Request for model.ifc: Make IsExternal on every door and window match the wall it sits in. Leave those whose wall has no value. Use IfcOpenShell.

First a look at what the model holds.

```python
import ifcopenshell
import ifcopenshell.util.element

model = ifcopenshell.open("model.ifc")
print(model.schema)
seen = {}
for e in model.by_type("IfcDoor") + model.by_type("IfcWindow"):
    if not e.FillsVoids:
        continue
    host = e.FillsVoids[0].RelatingOpeningElement.VoidsElements[0].RelatingBuildingElement
    own = ifcopenshell.util.element.get_pset(e, f"Pset_{e.is_a()[3:].removesuffix('StandardCase')}Common", "IsExternal")
    wall = ifcopenshell.util.element.get_pset(host, "Pset_WallCommon", "IsExternal")
    seen[e.is_a(), own, wall] = seen.get((e.is_a(), own, wall), 0) + 1
for (cls, own, wall), count in sorted(seen.items(), key=str):
    print(count, cls, "IsExternal:", own, "| host wall:", wall)
```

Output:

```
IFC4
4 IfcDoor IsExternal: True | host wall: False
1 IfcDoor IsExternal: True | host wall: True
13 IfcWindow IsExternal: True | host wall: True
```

```python
import ifcopenshell
import ifcopenshell.api.pset
import ifcopenshell.util.element

model = ifcopenshell.open("model.ifc")

count = 0
for ifc_class, pset_name in (("IfcDoor", "Pset_DoorCommon"), ("IfcWindow", "Pset_WindowCommon")):
    for e in model.by_type(ifc_class):
        if not e.FillsVoids:
            continue
        host = e.FillsVoids[0].RelatingOpeningElement.VoidsElements[0].RelatingBuildingElement
        external = ifcopenshell.util.element.get_pset(host, "Pset_WallCommon", "IsExternal")
        if external is None or ifcopenshell.util.element.get_pset(e, pset_name, "IsExternal") == external:
            continue
        pset = ifcopenshell.api.pset.add_pset(model, product=e, name=pset_name)
        ifcopenshell.api.pset.edit_pset(model, pset=pset, properties={"IsExternal": external})
        count += 1

print(count, "updated")

model.write("model-out.ifc")
```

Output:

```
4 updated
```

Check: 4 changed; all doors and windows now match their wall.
